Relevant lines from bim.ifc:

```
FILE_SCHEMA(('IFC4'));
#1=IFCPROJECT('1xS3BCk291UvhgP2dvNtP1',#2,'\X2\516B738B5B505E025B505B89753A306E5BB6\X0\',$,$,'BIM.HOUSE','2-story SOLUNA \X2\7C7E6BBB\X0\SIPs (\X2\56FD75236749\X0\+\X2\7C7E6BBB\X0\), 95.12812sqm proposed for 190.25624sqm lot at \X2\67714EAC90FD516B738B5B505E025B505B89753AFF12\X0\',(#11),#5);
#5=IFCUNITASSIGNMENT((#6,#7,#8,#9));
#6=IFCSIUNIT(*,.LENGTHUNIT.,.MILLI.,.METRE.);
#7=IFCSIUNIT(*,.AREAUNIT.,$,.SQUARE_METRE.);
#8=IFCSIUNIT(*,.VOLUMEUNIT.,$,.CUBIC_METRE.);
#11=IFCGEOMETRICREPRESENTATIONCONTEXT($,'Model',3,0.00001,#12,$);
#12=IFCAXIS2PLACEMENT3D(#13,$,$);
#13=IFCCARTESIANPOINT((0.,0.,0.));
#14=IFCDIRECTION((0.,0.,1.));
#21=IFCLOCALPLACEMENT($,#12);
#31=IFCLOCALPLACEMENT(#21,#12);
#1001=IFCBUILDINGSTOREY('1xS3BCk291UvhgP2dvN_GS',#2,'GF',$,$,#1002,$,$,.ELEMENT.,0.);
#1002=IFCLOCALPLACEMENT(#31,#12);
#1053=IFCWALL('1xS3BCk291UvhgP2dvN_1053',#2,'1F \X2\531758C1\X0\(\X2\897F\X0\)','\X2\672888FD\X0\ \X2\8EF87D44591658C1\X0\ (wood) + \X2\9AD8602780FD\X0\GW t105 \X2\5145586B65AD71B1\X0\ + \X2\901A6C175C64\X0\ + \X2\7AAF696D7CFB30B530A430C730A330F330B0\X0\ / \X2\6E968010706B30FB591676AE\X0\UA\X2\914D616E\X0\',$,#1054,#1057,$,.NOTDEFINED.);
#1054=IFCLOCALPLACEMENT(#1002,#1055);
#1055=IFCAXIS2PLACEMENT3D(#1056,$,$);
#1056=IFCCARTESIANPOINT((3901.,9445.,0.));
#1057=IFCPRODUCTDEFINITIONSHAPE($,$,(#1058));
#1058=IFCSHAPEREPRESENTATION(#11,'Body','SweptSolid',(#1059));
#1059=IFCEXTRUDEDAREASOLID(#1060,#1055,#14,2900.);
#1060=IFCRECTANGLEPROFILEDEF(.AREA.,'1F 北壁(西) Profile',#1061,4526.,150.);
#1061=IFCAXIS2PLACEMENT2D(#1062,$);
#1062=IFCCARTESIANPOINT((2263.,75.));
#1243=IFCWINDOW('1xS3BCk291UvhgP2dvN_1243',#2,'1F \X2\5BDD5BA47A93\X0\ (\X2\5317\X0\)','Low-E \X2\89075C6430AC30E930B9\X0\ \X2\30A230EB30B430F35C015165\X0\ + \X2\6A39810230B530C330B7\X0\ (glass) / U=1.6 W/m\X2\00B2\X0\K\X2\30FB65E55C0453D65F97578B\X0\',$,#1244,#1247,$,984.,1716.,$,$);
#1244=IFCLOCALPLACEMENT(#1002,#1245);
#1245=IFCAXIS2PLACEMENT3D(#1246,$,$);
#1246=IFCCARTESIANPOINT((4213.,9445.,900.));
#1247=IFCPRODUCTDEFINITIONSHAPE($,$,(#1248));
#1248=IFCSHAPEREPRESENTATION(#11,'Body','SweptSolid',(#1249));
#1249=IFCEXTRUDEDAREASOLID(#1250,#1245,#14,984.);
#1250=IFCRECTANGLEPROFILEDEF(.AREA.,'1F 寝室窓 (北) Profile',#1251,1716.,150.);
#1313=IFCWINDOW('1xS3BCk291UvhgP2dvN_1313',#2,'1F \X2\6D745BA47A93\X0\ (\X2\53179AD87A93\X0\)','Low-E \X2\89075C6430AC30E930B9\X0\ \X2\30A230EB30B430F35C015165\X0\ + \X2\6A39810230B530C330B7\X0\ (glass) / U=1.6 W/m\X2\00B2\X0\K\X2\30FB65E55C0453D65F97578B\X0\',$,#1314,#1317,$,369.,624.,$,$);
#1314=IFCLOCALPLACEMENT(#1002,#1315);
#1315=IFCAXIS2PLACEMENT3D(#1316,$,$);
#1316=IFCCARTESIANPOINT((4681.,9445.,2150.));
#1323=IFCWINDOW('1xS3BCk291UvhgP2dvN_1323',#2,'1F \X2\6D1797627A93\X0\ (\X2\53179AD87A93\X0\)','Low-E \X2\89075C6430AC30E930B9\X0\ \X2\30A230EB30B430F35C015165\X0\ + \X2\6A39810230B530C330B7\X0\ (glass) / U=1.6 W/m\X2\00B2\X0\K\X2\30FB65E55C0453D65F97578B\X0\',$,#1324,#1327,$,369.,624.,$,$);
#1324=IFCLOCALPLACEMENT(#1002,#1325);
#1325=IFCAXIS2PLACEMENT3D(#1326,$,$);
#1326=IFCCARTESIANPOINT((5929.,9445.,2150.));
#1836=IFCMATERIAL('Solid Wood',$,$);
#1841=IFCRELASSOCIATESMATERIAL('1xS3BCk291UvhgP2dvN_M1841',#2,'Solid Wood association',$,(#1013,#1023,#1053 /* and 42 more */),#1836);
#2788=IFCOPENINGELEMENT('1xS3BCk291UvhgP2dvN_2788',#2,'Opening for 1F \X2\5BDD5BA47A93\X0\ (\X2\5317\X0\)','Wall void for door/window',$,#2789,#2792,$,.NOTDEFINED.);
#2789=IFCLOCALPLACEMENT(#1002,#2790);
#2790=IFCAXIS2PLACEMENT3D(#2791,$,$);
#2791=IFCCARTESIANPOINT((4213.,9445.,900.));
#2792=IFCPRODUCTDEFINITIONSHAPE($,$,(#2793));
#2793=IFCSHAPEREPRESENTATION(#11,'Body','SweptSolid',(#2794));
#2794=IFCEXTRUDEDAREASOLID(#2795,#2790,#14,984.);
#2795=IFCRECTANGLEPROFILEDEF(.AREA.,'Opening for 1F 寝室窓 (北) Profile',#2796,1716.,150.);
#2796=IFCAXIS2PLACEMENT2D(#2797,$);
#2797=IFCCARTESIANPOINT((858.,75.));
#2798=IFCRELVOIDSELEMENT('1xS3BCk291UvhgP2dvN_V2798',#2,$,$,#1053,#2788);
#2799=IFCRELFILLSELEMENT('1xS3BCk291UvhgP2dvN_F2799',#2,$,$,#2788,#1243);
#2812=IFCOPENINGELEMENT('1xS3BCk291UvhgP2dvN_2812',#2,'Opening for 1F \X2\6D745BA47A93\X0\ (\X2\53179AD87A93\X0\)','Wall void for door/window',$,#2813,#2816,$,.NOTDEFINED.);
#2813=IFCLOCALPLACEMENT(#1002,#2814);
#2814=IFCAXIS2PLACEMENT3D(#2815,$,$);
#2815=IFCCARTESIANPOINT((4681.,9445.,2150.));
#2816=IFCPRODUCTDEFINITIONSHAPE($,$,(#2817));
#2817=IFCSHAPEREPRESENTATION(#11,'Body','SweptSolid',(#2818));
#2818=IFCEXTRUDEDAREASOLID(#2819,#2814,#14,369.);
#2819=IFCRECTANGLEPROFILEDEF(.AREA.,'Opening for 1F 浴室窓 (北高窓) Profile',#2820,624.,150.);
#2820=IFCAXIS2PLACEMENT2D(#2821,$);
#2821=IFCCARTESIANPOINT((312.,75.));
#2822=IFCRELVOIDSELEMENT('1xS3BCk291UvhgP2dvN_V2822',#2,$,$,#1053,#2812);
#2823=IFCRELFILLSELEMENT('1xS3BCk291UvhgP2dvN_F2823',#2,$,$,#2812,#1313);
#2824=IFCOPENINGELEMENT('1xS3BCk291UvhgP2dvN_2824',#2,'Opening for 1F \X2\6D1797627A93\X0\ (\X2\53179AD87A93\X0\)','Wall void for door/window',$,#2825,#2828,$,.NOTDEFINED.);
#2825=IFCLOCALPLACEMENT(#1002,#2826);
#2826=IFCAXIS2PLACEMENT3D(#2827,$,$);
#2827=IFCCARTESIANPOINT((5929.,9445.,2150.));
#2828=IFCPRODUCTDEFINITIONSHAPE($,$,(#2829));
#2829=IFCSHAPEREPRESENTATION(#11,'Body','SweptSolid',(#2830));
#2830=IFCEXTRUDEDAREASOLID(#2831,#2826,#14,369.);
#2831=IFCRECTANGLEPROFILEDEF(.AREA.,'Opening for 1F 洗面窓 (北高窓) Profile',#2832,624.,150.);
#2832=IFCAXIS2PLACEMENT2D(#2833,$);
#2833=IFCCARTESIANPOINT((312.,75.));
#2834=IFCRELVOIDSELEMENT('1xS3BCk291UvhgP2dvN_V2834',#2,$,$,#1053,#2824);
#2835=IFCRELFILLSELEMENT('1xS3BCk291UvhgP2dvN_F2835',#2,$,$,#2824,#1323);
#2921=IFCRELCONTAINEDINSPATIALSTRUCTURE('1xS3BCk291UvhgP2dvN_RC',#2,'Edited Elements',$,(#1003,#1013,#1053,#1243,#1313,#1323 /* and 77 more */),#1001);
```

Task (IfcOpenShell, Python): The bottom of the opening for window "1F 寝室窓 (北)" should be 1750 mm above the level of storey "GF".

```python
import numpy as np
import ifcopenshell
import ifcopenshell.api.geometry
import ifcopenshell.geom
import ifcopenshell.util.element
import ifcopenshell.util.placement
import ifcopenshell.util.shape
import ifcopenshell.util.unit

model = ifcopenshell.open("bim.ifc")
unit_scale = ifcopenshell.util.unit.calculate_unit_scale(model)

window = model.by_guid("1xS3BCk291UvhgP2dvN_1243")
opening = window.FillsVoids[0].RelatingOpeningElement
storey = ifcopenshell.util.element.get_container(window, ifc_class="IfcBuildingStorey")
level = ifcopenshell.util.placement.get_local_placement(storey.ObjectPlacement)[2, 3]

# The opening's origin need not be at the sill, so measure its lowest point.
shape = ifcopenshell.geom.create_shape(ifcopenshell.geom.settings(), opening)
bottom = ifcopenshell.util.shape.get_shape_bottom_elevation(shape, shape.geometry) / unit_scale
dz = level + 1.75 / unit_scale - bottom

shift = np.array([0.0, 0.0, dz])
# The window is not placed relative to its opening, so move both.
for product in (opening, window):
    matrix = ifcopenshell.util.placement.get_local_placement(product.ObjectPlacement)
    matrix[:3, 3] += shift
    ifcopenshell.api.geometry.edit_object_placement(model, product=product, matrix=matrix, is_si=False)

print(f"moved by {dz * unit_scale:+.3f} m")

model.write("bim_updated.ifc")
```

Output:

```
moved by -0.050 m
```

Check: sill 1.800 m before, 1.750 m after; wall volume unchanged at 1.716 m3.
